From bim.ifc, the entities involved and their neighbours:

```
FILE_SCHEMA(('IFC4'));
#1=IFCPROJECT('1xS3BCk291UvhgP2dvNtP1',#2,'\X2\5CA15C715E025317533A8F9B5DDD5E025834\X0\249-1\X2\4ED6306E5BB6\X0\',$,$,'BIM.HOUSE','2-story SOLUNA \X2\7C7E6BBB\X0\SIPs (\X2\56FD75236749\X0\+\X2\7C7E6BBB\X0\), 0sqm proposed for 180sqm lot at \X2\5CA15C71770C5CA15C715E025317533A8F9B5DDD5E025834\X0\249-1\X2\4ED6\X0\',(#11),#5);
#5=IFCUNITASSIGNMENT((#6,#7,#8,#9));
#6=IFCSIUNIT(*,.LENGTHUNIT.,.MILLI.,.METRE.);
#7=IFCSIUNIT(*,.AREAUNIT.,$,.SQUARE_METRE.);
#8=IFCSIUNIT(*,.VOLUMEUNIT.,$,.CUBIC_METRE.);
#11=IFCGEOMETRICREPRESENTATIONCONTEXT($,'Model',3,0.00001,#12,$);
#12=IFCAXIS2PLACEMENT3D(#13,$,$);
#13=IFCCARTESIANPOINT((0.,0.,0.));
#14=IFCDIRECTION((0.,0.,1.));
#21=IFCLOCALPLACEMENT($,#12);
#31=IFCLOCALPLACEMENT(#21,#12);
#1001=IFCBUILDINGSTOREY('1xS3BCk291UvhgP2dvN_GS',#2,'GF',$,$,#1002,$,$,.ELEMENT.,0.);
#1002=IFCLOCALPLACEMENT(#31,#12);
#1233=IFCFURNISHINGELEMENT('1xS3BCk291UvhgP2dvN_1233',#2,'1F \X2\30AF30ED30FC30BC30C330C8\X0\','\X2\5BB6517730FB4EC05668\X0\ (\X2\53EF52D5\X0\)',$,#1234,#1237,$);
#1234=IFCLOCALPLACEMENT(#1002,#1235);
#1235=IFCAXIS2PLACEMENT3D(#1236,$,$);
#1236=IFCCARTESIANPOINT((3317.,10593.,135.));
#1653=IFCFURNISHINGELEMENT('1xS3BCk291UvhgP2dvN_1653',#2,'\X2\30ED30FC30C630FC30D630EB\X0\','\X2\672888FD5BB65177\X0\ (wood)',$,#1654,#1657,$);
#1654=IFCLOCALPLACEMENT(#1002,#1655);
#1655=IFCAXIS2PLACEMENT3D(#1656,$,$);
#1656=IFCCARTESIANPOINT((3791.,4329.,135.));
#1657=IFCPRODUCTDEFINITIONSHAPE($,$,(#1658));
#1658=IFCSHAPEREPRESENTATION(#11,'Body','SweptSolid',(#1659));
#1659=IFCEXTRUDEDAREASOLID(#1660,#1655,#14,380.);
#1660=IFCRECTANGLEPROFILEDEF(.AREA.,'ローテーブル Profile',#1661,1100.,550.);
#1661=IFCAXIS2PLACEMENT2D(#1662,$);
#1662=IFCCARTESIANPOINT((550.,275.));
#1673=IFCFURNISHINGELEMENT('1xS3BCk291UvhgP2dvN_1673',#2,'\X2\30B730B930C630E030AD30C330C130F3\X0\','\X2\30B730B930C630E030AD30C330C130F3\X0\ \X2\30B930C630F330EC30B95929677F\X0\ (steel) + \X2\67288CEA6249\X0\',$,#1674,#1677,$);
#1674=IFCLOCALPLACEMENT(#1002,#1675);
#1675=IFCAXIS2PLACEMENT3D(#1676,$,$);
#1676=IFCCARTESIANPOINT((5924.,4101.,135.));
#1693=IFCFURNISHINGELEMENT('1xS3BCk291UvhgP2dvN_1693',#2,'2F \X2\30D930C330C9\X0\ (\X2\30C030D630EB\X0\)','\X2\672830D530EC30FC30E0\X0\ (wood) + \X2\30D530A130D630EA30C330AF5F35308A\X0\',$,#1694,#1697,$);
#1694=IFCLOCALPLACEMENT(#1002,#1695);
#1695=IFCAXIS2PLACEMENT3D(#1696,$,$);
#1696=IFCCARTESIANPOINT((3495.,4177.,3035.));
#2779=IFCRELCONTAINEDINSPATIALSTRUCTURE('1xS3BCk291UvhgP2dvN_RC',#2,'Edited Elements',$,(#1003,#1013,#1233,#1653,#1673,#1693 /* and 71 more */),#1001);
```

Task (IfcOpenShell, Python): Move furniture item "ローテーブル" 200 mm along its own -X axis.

```python
import ifcopenshell
import ifcopenshell.api.geometry
import ifcopenshell.util.placement
import ifcopenshell.util.unit

model = ifcopenshell.open("bim.ifc")
unit_scale = ifcopenshell.util.unit.calculate_unit_scale(model)

item = model.by_guid("1xS3BCk291UvhgP2dvN_1653")
matrix = ifcopenshell.util.placement.get_local_placement(item.ObjectPlacement)
matrix[:3, 3] -= matrix[:3, 0] * 0.2 / unit_scale
ifcopenshell.api.geometry.edit_object_placement(model, product=item, matrix=matrix, is_si=False)

print(ifcopenshell.util.placement.get_local_placement(item.ObjectPlacement).round(3) + 0.0)

model.write("bim_v2.ifc")
```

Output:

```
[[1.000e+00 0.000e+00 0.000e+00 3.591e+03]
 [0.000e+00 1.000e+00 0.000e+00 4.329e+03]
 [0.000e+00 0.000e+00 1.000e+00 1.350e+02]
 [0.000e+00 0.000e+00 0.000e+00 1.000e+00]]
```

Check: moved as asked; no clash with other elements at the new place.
